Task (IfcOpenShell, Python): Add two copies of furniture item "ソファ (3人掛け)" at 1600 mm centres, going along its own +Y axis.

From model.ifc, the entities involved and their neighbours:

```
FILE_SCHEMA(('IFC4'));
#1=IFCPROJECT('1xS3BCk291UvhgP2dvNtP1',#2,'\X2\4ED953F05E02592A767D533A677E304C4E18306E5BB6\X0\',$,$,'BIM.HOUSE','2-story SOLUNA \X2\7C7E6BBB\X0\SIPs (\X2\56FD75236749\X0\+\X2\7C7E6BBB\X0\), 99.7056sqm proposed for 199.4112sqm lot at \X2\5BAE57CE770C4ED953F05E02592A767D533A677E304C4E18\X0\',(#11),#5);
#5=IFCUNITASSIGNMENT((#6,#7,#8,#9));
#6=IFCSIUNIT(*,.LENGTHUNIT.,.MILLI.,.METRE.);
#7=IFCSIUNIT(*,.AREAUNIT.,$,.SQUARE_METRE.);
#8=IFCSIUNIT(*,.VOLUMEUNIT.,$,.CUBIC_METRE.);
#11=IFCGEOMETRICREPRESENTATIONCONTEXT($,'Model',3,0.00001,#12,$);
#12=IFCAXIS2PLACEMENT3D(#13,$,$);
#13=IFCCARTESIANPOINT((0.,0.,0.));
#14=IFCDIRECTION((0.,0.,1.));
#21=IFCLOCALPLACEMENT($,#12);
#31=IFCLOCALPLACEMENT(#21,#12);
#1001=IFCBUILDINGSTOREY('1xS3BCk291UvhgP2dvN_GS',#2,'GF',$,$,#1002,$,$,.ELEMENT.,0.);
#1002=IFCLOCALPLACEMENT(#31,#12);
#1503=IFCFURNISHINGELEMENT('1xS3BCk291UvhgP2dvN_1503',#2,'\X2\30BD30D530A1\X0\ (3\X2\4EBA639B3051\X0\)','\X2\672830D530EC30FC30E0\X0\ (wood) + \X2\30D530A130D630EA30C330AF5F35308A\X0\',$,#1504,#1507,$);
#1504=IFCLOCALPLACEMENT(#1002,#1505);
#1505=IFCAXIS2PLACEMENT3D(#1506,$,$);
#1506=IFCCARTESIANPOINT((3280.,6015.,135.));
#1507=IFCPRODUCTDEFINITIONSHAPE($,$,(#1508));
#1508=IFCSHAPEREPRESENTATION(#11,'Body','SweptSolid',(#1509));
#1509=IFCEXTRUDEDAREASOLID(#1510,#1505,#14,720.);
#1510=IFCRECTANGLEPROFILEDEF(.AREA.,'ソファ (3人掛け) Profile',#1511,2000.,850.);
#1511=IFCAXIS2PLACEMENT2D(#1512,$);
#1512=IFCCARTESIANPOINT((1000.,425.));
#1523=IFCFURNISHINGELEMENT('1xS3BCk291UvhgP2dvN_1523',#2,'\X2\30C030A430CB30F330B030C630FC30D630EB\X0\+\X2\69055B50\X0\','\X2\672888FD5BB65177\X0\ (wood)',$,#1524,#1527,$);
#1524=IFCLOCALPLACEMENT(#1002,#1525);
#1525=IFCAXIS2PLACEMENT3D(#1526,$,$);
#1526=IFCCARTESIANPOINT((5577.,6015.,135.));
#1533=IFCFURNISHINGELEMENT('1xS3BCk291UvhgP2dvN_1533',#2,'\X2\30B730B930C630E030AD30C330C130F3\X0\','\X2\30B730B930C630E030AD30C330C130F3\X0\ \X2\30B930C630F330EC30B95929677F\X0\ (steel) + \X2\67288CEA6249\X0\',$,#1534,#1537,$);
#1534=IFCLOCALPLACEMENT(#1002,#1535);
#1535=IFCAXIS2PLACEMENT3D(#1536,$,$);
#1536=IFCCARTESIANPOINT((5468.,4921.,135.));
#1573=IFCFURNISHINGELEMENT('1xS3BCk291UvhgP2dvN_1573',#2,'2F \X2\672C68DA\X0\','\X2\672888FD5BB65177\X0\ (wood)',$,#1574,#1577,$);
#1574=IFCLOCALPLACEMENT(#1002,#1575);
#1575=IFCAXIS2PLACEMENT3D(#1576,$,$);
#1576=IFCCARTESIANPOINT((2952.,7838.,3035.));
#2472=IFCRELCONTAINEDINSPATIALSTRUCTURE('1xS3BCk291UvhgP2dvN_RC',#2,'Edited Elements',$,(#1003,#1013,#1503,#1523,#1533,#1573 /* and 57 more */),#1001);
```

```python
import ifcopenshell
import ifcopenshell.api.geometry
import ifcopenshell.api.root
import ifcopenshell.util.element
import ifcopenshell.util.placement
import ifcopenshell.util.unit

model = ifcopenshell.open("model.ifc")
unit_scale = ifcopenshell.util.unit.calculate_unit_scale(model)


def reuse_history(source, copy):
    """copy_class also copies each property set's owner history, people and application; keep the originals."""
    for rel in copy.IsDefinedBy:
        if rel.is_a("IfcRelDefinesByProperties") and (history := rel.RelatingPropertyDefinition.OwnerHistory):
            rel.RelatingPropertyDefinition.OwnerHistory = source.OwnerHistory
            ifcopenshell.util.element.remove_deep2(model, history)


source = model.by_guid("1xS3BCk291UvhgP2dvN_1503")
base = ifcopenshell.util.placement.get_local_placement(source.ObjectPlacement)
step = base[:3, 1] * 1.6 / unit_scale

for i in range(1, 3):
    copy = ifcopenshell.api.root.copy_class(model, product=source)
    copy.Representation = ifcopenshell.util.element.copy_deep(
        model, source.Representation, exclude=["IfcGeometricRepresentationContext", "IfcRepresentationMap"]
    )
    reuse_history(source, copy)
    matrix = base.copy()
    matrix[:3, 3] += i * step
    print("added at", matrix[:3, 3].round(3) + 0.0)
    ifcopenshell.api.geometry.edit_object_placement(model, product=copy, matrix=matrix, is_si=False)

model.write("model_updated.ifc")
```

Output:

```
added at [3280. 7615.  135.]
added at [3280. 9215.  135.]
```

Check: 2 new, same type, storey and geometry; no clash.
